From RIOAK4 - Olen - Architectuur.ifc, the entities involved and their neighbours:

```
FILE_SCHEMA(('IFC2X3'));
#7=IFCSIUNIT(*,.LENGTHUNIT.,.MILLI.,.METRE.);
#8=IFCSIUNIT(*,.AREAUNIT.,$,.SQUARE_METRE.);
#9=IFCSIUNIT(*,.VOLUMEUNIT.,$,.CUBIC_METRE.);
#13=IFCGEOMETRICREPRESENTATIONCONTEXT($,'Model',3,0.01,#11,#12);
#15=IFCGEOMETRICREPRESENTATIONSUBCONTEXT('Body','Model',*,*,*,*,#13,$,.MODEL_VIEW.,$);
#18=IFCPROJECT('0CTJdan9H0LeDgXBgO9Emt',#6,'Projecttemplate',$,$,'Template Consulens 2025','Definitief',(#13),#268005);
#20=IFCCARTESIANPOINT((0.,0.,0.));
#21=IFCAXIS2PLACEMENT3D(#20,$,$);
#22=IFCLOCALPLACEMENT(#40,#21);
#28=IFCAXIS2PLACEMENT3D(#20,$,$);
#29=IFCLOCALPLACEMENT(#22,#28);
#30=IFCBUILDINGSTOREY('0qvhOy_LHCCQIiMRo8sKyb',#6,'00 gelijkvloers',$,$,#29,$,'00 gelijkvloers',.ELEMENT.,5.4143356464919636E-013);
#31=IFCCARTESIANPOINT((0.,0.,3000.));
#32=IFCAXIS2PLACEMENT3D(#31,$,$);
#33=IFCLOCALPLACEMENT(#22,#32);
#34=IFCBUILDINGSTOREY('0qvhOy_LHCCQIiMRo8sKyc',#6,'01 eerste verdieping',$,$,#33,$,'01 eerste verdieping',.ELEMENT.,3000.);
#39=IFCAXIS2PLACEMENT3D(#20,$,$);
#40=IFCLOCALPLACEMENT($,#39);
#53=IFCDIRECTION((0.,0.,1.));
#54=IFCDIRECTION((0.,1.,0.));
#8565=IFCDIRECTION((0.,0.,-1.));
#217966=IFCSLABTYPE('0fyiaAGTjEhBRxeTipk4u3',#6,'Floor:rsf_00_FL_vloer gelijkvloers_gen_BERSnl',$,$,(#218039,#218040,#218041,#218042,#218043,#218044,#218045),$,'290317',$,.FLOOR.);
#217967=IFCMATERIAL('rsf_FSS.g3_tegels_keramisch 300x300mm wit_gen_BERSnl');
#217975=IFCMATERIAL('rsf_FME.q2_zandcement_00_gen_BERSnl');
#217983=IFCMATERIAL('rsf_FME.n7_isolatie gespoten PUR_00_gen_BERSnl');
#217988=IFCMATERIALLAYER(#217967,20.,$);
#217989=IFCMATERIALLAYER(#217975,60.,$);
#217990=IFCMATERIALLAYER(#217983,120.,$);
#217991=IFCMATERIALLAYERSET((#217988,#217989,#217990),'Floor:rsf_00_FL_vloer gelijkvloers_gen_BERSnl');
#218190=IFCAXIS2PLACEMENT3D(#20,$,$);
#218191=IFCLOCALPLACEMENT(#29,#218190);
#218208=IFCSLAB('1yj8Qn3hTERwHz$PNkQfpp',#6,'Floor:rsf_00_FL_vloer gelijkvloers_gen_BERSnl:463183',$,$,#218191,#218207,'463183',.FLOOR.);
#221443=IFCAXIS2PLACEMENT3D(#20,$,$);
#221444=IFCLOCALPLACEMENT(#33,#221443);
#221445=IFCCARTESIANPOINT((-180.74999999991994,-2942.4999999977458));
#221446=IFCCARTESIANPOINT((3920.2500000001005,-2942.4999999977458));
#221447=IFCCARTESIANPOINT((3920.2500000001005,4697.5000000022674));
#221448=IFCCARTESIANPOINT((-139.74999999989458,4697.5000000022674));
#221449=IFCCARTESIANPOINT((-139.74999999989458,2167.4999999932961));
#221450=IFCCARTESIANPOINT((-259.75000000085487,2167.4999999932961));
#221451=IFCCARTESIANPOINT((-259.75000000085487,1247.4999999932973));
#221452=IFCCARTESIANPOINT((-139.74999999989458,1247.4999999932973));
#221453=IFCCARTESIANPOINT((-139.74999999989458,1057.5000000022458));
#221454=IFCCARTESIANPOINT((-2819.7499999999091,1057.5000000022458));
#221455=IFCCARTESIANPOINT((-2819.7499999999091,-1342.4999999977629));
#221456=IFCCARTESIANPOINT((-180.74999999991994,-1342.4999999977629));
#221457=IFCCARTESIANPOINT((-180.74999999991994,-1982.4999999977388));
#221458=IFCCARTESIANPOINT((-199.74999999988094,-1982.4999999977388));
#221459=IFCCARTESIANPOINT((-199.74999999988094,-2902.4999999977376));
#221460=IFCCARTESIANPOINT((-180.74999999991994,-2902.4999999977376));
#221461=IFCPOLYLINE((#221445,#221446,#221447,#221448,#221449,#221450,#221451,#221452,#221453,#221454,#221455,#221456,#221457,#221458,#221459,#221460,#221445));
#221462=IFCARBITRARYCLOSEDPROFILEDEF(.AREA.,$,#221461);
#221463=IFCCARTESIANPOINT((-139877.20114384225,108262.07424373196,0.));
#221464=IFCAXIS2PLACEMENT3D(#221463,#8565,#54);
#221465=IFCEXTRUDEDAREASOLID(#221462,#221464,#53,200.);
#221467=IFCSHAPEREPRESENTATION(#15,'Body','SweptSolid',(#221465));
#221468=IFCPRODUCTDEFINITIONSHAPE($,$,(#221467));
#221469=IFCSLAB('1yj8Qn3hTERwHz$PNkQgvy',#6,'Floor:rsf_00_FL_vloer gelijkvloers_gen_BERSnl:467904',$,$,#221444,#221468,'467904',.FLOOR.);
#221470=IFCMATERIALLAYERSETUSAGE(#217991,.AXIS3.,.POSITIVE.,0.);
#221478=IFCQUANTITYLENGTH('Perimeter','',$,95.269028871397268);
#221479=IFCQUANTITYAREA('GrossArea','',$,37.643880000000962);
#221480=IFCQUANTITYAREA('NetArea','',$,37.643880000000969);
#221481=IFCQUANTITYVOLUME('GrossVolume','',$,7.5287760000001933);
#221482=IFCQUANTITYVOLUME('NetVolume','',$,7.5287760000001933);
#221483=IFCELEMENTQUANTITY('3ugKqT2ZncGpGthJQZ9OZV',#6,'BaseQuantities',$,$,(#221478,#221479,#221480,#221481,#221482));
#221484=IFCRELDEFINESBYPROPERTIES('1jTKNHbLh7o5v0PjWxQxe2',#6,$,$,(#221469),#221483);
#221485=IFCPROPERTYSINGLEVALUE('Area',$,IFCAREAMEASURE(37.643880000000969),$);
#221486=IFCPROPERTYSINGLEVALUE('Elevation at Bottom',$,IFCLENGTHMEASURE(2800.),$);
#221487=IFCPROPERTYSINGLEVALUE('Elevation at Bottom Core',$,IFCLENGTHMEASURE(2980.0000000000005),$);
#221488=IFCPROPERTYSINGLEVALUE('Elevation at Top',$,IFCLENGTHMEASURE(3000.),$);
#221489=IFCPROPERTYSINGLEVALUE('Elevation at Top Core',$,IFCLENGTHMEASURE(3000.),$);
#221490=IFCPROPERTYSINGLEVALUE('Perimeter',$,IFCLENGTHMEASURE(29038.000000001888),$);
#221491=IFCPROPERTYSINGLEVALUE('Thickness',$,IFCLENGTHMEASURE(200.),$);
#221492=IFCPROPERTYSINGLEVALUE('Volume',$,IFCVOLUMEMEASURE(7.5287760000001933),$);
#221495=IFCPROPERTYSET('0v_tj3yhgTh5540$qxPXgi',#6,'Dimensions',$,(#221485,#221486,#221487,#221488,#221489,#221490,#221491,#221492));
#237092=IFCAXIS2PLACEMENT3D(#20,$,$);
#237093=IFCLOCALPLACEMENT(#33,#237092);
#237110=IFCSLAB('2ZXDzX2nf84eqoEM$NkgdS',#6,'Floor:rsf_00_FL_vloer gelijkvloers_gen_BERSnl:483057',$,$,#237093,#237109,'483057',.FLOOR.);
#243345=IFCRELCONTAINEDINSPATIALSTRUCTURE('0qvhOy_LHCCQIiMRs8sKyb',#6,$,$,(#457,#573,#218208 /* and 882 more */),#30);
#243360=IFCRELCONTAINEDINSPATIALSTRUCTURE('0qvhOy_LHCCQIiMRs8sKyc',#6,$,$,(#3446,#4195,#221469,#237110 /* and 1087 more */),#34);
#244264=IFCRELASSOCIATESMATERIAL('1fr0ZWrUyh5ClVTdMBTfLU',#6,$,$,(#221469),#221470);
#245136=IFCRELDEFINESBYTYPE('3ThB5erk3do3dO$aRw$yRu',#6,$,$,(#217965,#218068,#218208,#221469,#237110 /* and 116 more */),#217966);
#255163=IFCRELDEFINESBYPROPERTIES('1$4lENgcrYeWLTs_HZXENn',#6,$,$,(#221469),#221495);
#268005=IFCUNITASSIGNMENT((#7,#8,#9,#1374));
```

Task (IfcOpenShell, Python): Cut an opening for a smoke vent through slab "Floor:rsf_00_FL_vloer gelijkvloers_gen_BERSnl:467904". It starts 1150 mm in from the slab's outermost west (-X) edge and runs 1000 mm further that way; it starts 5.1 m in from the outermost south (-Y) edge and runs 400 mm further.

```python
import numpy as np
import ifcopenshell
import ifcopenshell.api.feature
import ifcopenshell.api.geometry
import ifcopenshell.api.pset
import ifcopenshell.api.root
import ifcopenshell.geom
import ifcopenshell.util.element
import ifcopenshell.util.placement
import ifcopenshell.util.representation
import ifcopenshell.util.shape
import ifcopenshell.util.unit

model = ifcopenshell.open("RIOAK4 - Olen - Architectuur.ifc")
unit_scale = ifcopenshell.util.unit.calculate_unit_scale(model)
area_scale = ifcopenshell.util.unit.calculate_unit_scale(model, "AREAUNIT")
volume_scale = ifcopenshell.util.unit.calculate_unit_scale(model, "VOLUMEUNIT")
settings = ifcopenshell.geom.settings()


def volume(element):
    """Net volume in cubic metres, openings subtracted."""
    shape = ifcopenshell.geom.create_shape(settings, element)
    return ifcopenshell.util.shape.get_volume(shape.geometry)


slab = model.by_id(221469)
before = volume(slab)

# Extent in the slab's own axes, in metres. The edges named are its -X and -Y sides.
slab_shape = ifcopenshell.geom.create_shape(settings, slab)
vertices = ifcopenshell.util.shape.get_vertices(slab_shape.geometry)
x_min, y_min, bottom = vertices.min(axis=0)
top = vertices[:, 2].max()

opening = ifcopenshell.api.root.create_entity(model, ifc_class="IfcOpeningElement", name="Smoke vent opening")
context = ifcopenshell.util.representation.get_context(model, "Model", "Body", "MODEL_VIEW")
width, depth = 1, 0.4
outline = [(0.0, 0.0), (width, 0.0), (width, depth), (0.0, depth), (0.0, 0.0)]
# Overshoot both faces by 50 mm so the cut is clean.
shape = ifcopenshell.api.geometry.add_slab_representation(
    model, context=context, depth=top - bottom + 0.1, polyline=outline
)
ifcopenshell.api.geometry.assign_representation(model, product=opening, representation=shape)

matrix = ifcopenshell.util.placement.get_local_placement(slab.ObjectPlacement)
matrix[:, 3] = matrix @ np.append(np.array([x_min + 1.15, y_min + 5.1, bottom - 0.05]) / unit_scale, 1.0)
ifcopenshell.api.geometry.edit_object_placement(model, product=opening, matrix=matrix, is_si=False)
ifcopenshell.api.feature.add_feature(model, feature=opening, element=slab)

after = volume(slab)

# Update the slab's stored quantities.
qto = model.by_id(ifcopenshell.util.element.get_pset(slab, "BaseQuantities", should_inherit=False)["id"])
ifcopenshell.api.pset.edit_qto(model, qto=qto, properties={
    "NetArea": after / (top - bottom) / area_scale,
    "NetVolume": after / volume_scale,
})
pset = model.by_id(ifcopenshell.util.element.get_pset(slab, "Dimensions", should_inherit=False)["id"])
ifcopenshell.api.pset.edit_pset(model, pset=pset, properties={
    "Area": model.create_entity("IfcAreaMeasure", after / (top - bottom) / area_scale),
    "Volume": model.create_entity("IfcVolumeMeasure", after / volume_scale),
})

print(f"slab volume {before:.3f} -> {after:.3f} m3")

model.write("RIOAK4 - Olen - Architectuur_rev.ifc")
```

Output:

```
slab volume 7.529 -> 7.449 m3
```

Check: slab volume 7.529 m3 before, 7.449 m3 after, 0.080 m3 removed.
